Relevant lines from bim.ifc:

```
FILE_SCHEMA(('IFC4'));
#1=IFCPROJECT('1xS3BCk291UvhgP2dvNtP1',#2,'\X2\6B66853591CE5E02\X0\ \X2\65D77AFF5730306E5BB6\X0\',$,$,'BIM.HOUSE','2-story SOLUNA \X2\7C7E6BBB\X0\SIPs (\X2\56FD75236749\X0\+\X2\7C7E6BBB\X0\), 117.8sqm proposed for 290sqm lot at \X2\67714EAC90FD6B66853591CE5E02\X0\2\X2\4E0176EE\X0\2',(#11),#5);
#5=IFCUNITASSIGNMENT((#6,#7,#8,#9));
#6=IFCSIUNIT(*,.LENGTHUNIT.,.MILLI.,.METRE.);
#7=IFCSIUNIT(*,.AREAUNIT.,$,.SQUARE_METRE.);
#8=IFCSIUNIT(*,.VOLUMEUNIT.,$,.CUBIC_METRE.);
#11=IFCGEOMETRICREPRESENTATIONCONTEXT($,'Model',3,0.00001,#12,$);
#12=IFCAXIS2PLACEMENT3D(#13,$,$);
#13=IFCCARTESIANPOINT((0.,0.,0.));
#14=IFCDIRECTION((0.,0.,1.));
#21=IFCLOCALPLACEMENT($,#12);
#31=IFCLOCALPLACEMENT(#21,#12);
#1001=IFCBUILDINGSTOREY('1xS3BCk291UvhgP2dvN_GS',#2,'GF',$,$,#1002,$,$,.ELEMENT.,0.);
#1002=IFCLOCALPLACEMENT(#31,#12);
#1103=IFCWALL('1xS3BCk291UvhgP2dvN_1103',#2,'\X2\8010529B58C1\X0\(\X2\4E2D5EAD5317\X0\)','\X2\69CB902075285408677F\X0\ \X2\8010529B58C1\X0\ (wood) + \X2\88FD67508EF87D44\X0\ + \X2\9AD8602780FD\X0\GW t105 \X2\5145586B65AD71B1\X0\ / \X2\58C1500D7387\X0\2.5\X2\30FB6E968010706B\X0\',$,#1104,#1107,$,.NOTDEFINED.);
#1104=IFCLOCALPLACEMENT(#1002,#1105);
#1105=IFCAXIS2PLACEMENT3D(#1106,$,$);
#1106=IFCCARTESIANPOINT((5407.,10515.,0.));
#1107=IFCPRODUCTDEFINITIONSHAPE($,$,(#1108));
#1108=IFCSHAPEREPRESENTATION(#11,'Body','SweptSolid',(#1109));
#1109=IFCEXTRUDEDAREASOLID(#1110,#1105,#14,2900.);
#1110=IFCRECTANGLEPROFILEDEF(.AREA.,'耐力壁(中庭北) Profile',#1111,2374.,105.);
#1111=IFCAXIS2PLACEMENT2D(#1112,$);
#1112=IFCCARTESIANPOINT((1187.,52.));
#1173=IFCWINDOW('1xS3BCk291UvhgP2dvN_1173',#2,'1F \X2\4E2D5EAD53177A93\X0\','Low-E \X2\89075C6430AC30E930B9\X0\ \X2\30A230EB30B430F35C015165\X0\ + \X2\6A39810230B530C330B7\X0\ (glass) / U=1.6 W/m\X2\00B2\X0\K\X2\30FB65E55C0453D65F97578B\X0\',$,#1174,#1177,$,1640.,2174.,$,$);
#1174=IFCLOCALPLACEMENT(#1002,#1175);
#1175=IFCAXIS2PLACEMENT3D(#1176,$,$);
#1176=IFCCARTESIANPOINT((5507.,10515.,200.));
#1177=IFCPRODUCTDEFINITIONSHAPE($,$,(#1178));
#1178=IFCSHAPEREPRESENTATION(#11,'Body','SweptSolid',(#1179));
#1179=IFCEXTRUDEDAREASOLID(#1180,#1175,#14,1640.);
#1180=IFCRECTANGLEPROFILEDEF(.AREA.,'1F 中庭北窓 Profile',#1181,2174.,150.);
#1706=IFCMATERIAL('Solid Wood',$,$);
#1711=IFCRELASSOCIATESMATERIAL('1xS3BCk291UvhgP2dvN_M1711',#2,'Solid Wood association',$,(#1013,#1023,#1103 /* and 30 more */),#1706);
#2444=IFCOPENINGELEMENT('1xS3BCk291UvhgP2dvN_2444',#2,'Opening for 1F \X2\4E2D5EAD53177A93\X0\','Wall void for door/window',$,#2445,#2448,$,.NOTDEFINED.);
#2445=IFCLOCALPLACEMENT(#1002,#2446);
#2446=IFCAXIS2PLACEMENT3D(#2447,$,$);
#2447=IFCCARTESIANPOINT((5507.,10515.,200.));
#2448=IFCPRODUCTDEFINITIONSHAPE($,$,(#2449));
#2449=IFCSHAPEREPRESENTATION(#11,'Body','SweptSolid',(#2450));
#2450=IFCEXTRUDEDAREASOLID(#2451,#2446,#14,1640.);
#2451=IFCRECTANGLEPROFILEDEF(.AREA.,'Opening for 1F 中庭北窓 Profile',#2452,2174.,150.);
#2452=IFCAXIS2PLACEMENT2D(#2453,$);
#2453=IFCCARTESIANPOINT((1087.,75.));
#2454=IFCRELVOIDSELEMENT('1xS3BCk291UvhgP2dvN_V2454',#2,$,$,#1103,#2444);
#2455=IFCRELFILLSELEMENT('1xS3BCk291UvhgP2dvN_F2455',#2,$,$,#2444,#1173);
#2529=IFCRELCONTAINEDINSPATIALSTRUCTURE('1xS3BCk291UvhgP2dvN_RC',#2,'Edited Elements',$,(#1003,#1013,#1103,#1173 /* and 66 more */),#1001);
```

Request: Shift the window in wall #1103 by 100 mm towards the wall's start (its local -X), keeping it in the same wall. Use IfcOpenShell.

```python
import ifcopenshell
import ifcopenshell.api.geometry
import ifcopenshell.util.placement

model = ifcopenshell.open("bim.ifc")

window = model.by_guid("1xS3BCk291UvhgP2dvN_1173")
opening = window.FillsVoids[0].RelatingOpeningElement
wall = opening.VoidsElements[0].RelatingBuildingElement

wall_matrix = ifcopenshell.util.placement.get_local_placement(wall.ObjectPlacement)
shift = wall_matrix[:3, 0] * -100.0
before = ifcopenshell.util.placement.get_local_placement(window.ObjectPlacement)[:3, 3].copy()

# The window is not placed relative to its opening, so move both.
for product in (opening, window):
    matrix = ifcopenshell.util.placement.get_local_placement(product.ObjectPlacement)
    matrix[:3, 3] += shift
    ifcopenshell.api.geometry.edit_object_placement(model, product=product, matrix=matrix, is_si=False)

after = ifcopenshell.util.placement.get_local_placement(window.ObjectPlacement)[:3, 3]
print("window moved by", (after - before).round(3) + 0.0)

model.write("bim-out.ifc")
```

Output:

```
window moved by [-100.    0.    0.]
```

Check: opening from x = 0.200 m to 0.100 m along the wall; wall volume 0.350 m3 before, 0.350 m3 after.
